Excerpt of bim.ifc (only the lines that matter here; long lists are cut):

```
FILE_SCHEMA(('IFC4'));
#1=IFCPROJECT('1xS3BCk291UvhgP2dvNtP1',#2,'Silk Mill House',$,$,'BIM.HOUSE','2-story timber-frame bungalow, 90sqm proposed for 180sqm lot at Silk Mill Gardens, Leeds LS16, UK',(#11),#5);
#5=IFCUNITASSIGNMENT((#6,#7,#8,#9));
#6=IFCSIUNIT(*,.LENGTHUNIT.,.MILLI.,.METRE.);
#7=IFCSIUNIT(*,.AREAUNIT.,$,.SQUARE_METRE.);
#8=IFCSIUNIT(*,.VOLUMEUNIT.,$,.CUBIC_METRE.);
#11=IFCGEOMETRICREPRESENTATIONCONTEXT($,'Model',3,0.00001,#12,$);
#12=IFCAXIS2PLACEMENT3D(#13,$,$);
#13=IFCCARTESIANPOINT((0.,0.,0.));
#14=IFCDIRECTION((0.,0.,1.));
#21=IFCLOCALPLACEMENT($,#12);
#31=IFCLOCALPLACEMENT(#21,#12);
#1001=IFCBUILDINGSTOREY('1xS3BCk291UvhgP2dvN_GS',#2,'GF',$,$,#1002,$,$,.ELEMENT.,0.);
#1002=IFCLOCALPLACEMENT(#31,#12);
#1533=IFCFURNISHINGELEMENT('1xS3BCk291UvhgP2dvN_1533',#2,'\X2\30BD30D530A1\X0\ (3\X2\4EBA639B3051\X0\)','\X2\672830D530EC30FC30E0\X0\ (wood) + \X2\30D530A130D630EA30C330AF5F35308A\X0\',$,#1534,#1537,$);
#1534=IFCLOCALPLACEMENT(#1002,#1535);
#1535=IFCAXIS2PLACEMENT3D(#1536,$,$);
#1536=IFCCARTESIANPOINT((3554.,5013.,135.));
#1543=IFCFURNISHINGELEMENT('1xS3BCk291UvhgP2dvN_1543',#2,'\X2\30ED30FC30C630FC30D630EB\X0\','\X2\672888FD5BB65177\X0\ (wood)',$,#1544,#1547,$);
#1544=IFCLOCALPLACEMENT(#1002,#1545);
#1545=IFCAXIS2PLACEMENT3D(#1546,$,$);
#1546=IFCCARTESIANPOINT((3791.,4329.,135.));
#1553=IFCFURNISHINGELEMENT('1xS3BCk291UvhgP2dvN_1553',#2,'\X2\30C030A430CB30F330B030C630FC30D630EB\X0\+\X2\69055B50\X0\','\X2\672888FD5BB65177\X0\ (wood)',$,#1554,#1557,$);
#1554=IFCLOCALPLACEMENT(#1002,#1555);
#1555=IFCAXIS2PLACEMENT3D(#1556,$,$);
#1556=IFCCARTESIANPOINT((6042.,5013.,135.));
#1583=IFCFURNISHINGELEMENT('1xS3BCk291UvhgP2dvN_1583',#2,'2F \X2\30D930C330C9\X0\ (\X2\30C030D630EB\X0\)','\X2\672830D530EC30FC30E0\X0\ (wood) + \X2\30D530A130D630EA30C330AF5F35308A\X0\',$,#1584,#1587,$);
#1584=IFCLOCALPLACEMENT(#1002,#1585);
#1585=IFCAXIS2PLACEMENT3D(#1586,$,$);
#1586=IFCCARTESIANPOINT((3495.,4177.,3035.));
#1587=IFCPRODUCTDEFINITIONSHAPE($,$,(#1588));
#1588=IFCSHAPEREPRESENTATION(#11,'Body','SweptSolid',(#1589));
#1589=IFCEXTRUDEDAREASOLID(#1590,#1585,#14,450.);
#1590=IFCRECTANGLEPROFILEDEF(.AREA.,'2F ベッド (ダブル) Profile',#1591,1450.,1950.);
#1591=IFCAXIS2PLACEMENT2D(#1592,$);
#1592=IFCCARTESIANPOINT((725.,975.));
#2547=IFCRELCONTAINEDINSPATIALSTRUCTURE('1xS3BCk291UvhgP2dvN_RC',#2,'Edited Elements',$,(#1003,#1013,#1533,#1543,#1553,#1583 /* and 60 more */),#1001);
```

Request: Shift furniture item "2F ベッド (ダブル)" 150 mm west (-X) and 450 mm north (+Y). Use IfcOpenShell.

```python
import ifcopenshell
import ifcopenshell.api.geometry
import ifcopenshell.util.placement
import ifcopenshell.util.unit

model = ifcopenshell.open("bim.ifc")
unit_scale = ifcopenshell.util.unit.calculate_unit_scale(model)

item = model.by_guid("1xS3BCk291UvhgP2dvN_1583")
matrix = ifcopenshell.util.placement.get_local_placement(item.ObjectPlacement)
matrix[0, 3] -= 0.15 / unit_scale
matrix[1, 3] += 0.45 / unit_scale
ifcopenshell.api.geometry.edit_object_placement(model, product=item, matrix=matrix, is_si=False)

print(ifcopenshell.util.placement.get_local_placement(item.ObjectPlacement).round(3) + 0.0)

model.write("bim_rev.ifc")
```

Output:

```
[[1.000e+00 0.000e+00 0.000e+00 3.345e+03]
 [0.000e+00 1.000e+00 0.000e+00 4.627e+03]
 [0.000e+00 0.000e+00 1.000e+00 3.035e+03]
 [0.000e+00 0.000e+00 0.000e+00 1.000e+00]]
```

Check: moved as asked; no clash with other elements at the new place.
